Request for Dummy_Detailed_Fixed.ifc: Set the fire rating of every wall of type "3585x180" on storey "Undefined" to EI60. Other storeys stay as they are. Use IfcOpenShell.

First a look at what the model holds.

```python
import ifcopenshell
import ifcopenshell.util.element

model = ifcopenshell.open("Dummy_Detailed_Fixed.ifc")
print(model.schema)
storey = next(s for s in model.by_type("IfcBuildingStorey") if s.Name == "Undefined")
walls = [e for e in ifcopenshell.util.element.get_decomposition(storey) if e.is_a("IfcWall")]
seen = {}
for e in walls:
    element_type = ifcopenshell.util.element.get_type(e)
    key = (element_type.Name if element_type != e and element_type else None, ifcopenshell.util.element.get_pset(e, "Pset_WallCommon", "FireRating"))
    seen[key] = seen.get(key, 0) + 1
for (name, value), count in sorted(seen.items(), key=str):
    print(count, "x", name, "|", value)
```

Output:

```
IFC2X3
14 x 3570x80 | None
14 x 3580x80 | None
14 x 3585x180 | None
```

```python
import ifcopenshell
import ifcopenshell.api.pset
import ifcopenshell.util.element

model = ifcopenshell.open("Dummy_Detailed_Fixed.ifc")

storey = next(s for s in model.by_type("IfcBuildingStorey") if s.Name == "Undefined")
walls = [e for e in ifcopenshell.util.element.get_decomposition(storey) if e.is_a("IfcWall")]

count = 0
for e in walls:
    element_type = ifcopenshell.util.element.get_type(e)
    if element_type in (None, e) or element_type.Name != "3585x180":
        continue
    found = ifcopenshell.util.element.get_pset(e, "Pset_WallCommon", should_inherit=False)
    if found:
        pset = model.by_id(found["id"])
        if len(ifcopenshell.util.element.get_elements_by_pset(pset)) > 1:
            pset = ifcopenshell.api.pset.unshare_pset(model, products=[e], pset=pset)[0]
    else:
        pset = ifcopenshell.api.pset.add_pset(model, product=e, name="Pset_WallCommon")
    ifcopenshell.api.pset.edit_pset(model, pset=pset, properties={"FireRating": "EI60"})
    count += 1

print(count, "walls updated")

model.write("Dummy_Detailed_Fixed-out.ifc")
```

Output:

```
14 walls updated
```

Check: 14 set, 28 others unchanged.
